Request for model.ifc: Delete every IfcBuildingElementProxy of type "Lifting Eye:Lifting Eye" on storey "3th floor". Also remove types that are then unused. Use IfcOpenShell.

First a look at what the model holds.

```python
import ifcopenshell
import ifcopenshell.util.element

model = ifcopenshell.open("model.ifc")
print(model.schema)
storey = next(s for s in model.by_type("IfcBuildingStorey") if s.Name == "3th floor")
proxies = [e for e in ifcopenshell.util.element.get_decomposition(storey) if e.is_a("IfcBuildingElementProxy")]
seen = {}
for e in proxies:
    element_type = ifcopenshell.util.element.get_type(e)
    name = element_type.Name if element_type not in (None, e) else None
    seen[name] = seen.get(name, 0) + 1
for name, count in sorted(seen.items(), key=str):
    print(count, "x", name)
```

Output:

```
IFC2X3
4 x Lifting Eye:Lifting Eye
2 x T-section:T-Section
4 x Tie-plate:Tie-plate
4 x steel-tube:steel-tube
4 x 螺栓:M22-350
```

```python
import ifcopenshell
import ifcopenshell.api.root
import ifcopenshell.util.element

model = ifcopenshell.open("model.ifc")

storey = next(s for s in model.by_type("IfcBuildingStorey") if s.Name == "3th floor")
proxies = [e for e in ifcopenshell.util.element.get_decomposition(storey) if e.is_a("IfcBuildingElementProxy")]
targets = [e for e in proxies if (t := ifcopenshell.util.element.get_type(e)) not in (None, e) and t.Name == "Lifting Eye:Lifting Eye"]
types = {ifcopenshell.util.element.get_type(e) for e in targets} - {None, *targets}

for e in targets:
    ifcopenshell.api.root.remove_product(model, product=e)
print(len(targets), "removed")

unused = [t for t in types if not ifcopenshell.util.element.get_types(t)]
for t in unused:
    ifcopenshell.api.root.remove_product(model, product=t)
print(len(unused), "unused types removed")

model.write("model-out.ifc")
```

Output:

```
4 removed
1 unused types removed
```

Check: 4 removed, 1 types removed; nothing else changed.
